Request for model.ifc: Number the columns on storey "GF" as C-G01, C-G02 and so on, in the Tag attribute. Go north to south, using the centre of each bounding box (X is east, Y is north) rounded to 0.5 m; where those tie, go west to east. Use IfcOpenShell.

First a look at what the model holds.

```python
import ifcopenshell
import ifcopenshell.util.element
import ifcopenshell.util.placement

model = ifcopenshell.open("model.ifc")
print(model.schema)
storey = next(s for s in model.by_type("IfcBuildingStorey") if s.Name == "GF")
columns = [e for e in ifcopenshell.util.element.get_decomposition(storey) if e.is_a("IfcColumn")]
for e in sorted(columns, key=lambda e: e.id()):
    origin = ifcopenshell.util.placement.get_local_placement(e.ObjectPlacement)[:3, 3]
    print(e.id(), e.Tag, e.Name, origin.round(2) + 0.0, sep=" | ")
```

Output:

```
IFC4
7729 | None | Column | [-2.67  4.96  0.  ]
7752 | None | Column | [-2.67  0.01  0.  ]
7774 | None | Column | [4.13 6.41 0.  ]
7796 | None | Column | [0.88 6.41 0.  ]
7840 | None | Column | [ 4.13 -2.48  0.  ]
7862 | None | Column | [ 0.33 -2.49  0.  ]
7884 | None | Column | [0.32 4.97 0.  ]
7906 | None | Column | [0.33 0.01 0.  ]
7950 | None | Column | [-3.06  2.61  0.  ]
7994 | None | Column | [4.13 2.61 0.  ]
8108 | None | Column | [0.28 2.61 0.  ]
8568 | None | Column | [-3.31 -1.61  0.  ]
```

```python
import ifcopenshell
import ifcopenshell.geom
import ifcopenshell.util.element
import ifcopenshell.util.shape

model = ifcopenshell.open("model.ifc")
settings = ifcopenshell.geom.settings()
settings.set("use-world-coords", True)


def centre(element):
    shape = ifcopenshell.geom.create_shape(settings, element)
    return ifcopenshell.util.shape.get_bbox_centroid(shape.geometry)


storey = next(s for s in model.by_type("IfcBuildingStorey") if s.Name == "GF")
columns = [e for e in ifcopenshell.util.element.get_decomposition(storey) if e.is_a("IfcColumn")]

# Insertion points can sit at a corner or the storey origin, so sort by the geometry (in metres).
centres = {e: centre(e) for e in columns}
columns.sort(key=lambda e: (-round(centres[e][1] / 0.5), centres[e][0]))

for i, e in enumerate(columns, start=1):
    number = f"C-G{i:02d}"
    e.Tag = number
    print(e.id(), number)

model.write("model_edited.ifc")
```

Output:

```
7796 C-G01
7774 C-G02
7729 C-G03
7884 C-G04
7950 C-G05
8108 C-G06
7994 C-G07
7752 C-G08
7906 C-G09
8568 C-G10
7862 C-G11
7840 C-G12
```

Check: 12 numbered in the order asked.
